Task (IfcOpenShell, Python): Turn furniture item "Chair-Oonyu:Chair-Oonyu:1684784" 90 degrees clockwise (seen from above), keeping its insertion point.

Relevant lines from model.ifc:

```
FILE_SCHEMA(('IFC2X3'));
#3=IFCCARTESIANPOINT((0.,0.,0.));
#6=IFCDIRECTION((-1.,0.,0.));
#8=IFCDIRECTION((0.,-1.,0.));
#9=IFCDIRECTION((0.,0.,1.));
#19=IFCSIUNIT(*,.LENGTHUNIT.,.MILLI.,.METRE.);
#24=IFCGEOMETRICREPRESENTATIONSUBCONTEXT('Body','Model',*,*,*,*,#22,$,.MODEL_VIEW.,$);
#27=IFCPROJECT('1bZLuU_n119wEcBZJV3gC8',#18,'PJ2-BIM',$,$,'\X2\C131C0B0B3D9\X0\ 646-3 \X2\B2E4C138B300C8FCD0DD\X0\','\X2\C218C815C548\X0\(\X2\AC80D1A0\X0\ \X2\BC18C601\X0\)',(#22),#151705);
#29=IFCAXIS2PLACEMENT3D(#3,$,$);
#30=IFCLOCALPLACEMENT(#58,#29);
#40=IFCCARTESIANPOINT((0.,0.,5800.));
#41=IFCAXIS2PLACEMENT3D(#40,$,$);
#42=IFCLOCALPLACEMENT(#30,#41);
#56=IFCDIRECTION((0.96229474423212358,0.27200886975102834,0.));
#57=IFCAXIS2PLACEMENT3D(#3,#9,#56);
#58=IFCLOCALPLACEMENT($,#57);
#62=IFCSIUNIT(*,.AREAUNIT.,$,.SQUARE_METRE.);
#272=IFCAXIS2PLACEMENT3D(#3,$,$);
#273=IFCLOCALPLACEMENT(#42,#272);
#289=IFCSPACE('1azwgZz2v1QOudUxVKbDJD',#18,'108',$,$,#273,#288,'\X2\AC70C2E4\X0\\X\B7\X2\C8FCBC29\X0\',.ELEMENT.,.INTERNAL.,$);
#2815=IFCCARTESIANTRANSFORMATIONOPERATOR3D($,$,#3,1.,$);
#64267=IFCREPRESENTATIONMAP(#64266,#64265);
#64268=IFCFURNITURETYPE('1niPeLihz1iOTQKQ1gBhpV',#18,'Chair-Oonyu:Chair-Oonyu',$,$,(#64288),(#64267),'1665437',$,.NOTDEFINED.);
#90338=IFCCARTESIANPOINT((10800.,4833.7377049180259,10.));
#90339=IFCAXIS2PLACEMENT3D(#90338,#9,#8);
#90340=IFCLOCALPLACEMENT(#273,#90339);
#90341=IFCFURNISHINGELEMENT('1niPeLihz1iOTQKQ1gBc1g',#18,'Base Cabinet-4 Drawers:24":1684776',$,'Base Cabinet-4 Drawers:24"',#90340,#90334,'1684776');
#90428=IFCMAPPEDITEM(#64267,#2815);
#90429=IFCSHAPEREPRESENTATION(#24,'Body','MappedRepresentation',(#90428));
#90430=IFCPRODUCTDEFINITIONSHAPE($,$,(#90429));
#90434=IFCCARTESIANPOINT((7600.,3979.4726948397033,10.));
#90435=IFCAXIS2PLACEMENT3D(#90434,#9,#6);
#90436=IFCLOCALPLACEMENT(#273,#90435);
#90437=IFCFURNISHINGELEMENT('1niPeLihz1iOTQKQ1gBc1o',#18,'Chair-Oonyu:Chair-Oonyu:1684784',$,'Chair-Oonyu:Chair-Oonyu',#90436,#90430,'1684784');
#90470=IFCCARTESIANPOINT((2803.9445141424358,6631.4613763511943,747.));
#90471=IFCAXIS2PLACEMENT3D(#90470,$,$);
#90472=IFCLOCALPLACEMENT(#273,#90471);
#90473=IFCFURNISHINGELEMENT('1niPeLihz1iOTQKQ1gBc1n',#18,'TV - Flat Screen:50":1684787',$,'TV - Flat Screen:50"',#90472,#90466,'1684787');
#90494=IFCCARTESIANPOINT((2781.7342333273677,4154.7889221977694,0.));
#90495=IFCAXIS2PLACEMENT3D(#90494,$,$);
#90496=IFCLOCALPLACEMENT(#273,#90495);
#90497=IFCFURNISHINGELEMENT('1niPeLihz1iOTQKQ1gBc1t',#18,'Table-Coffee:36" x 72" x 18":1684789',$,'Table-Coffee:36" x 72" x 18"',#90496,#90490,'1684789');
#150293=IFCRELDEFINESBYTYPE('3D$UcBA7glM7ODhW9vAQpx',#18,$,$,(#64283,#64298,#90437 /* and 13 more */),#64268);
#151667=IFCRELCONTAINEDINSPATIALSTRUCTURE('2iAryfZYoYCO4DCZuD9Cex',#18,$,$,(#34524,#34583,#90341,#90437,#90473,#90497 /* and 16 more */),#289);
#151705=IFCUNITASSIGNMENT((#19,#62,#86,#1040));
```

```python
import ifcopenshell
import ifcopenshell.api.geometry
import ifcopenshell.util.placement

model = ifcopenshell.open("model.ifc")

item = model.by_guid("1niPeLihz1iOTQKQ1gBc1o")
matrix = ifcopenshell.util.placement.get_local_placement(item.ObjectPlacement)
matrix = matrix @ ifcopenshell.util.placement.rotation(-90, "Z")
ifcopenshell.api.geometry.edit_object_placement(model, product=item, matrix=matrix, is_si=False)

print(ifcopenshell.util.placement.get_local_placement(item.ObjectPlacement).round(3) + 0.0)

model.write("model_v2.ifc")
```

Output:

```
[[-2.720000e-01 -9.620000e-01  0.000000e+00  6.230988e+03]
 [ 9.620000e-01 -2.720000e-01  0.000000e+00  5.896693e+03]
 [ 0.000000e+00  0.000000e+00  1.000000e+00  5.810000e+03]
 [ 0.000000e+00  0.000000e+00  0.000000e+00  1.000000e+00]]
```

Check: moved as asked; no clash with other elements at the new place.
